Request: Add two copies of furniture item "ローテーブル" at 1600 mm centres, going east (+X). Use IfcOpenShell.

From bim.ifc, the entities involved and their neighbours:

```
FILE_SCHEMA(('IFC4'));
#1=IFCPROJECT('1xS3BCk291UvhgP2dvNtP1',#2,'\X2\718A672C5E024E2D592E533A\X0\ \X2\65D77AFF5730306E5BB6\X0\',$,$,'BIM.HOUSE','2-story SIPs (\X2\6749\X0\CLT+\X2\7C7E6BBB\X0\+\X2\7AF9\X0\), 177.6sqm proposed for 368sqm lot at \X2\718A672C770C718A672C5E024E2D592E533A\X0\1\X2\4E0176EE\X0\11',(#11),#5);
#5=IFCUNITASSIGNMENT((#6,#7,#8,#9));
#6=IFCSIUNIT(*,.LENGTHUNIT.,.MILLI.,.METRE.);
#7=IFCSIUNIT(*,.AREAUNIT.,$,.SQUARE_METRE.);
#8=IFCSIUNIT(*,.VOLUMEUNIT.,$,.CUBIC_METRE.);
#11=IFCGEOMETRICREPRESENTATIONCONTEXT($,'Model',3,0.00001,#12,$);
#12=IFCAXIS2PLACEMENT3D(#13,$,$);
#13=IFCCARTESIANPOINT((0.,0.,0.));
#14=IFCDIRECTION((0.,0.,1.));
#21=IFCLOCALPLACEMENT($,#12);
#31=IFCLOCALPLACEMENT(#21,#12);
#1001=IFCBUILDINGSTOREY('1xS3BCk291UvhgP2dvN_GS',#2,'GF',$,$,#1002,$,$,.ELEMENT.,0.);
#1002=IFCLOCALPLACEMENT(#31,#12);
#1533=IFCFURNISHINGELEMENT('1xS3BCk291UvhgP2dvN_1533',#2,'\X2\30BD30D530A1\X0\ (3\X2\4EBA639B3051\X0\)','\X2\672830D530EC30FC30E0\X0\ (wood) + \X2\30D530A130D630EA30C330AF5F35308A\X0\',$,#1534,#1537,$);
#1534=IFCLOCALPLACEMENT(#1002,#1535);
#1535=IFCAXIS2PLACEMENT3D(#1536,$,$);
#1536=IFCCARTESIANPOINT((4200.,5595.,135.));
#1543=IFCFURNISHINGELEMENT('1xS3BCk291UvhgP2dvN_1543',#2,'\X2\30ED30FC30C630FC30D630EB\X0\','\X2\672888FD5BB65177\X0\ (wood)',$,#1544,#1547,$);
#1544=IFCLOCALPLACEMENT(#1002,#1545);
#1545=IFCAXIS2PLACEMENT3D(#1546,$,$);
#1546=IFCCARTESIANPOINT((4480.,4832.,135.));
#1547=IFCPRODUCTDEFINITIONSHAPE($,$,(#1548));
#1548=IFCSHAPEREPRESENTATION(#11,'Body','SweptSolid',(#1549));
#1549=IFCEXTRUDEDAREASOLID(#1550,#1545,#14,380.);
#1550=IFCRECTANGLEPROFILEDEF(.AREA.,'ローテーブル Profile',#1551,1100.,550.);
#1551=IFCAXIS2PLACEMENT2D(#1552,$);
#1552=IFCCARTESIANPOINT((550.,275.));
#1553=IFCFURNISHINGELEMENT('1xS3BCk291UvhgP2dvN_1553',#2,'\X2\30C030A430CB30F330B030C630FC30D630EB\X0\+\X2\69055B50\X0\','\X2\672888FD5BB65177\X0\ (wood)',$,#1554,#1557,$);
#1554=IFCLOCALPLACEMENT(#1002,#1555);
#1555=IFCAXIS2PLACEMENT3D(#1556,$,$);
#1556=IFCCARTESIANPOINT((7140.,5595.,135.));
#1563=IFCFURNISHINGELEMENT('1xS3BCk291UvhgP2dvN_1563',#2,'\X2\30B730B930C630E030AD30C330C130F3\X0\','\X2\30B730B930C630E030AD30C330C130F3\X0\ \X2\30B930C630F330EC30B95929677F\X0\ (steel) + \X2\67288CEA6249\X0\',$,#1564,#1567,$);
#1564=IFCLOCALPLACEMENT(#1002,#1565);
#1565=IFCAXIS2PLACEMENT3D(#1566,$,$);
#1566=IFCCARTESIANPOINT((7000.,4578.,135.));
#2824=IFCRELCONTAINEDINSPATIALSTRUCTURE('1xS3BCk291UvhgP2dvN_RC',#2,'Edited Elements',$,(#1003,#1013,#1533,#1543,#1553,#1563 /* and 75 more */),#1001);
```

```python
import numpy as np
import ifcopenshell
import ifcopenshell.api.geometry
import ifcopenshell.api.root
import ifcopenshell.util.element
import ifcopenshell.util.placement
import ifcopenshell.util.unit

model = ifcopenshell.open("bim.ifc")
unit_scale = ifcopenshell.util.unit.calculate_unit_scale(model)


def reuse_history(source, copy):
    """copy_class also copies each property set's owner history, people and application; keep the originals."""
    for rel in copy.IsDefinedBy:
        if rel.is_a("IfcRelDefinesByProperties") and (history := rel.RelatingPropertyDefinition.OwnerHistory):
            rel.RelatingPropertyDefinition.OwnerHistory = source.OwnerHistory
            ifcopenshell.util.element.remove_deep2(model, history)


source = model.by_id(1543)
base = ifcopenshell.util.placement.get_local_placement(source.ObjectPlacement)
step = np.array([1.0, 0.0, 0.0]) * 1.6 / unit_scale

for i in range(1, 3):
    copy = ifcopenshell.api.root.copy_class(model, product=source)
    copy.Representation = ifcopenshell.util.element.copy_deep(
        model, source.Representation, exclude=["IfcGeometricRepresentationContext", "IfcRepresentationMap"]
    )
    reuse_history(source, copy)
    matrix = base.copy()
    matrix[:3, 3] += i * step
    print("added at", matrix[:3, 3].round(3) + 0.0)
    ifcopenshell.api.geometry.edit_object_placement(model, product=copy, matrix=matrix, is_si=False)

model.write("bim_edited.ifc")
```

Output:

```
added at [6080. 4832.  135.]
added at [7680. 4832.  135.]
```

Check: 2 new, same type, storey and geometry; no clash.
